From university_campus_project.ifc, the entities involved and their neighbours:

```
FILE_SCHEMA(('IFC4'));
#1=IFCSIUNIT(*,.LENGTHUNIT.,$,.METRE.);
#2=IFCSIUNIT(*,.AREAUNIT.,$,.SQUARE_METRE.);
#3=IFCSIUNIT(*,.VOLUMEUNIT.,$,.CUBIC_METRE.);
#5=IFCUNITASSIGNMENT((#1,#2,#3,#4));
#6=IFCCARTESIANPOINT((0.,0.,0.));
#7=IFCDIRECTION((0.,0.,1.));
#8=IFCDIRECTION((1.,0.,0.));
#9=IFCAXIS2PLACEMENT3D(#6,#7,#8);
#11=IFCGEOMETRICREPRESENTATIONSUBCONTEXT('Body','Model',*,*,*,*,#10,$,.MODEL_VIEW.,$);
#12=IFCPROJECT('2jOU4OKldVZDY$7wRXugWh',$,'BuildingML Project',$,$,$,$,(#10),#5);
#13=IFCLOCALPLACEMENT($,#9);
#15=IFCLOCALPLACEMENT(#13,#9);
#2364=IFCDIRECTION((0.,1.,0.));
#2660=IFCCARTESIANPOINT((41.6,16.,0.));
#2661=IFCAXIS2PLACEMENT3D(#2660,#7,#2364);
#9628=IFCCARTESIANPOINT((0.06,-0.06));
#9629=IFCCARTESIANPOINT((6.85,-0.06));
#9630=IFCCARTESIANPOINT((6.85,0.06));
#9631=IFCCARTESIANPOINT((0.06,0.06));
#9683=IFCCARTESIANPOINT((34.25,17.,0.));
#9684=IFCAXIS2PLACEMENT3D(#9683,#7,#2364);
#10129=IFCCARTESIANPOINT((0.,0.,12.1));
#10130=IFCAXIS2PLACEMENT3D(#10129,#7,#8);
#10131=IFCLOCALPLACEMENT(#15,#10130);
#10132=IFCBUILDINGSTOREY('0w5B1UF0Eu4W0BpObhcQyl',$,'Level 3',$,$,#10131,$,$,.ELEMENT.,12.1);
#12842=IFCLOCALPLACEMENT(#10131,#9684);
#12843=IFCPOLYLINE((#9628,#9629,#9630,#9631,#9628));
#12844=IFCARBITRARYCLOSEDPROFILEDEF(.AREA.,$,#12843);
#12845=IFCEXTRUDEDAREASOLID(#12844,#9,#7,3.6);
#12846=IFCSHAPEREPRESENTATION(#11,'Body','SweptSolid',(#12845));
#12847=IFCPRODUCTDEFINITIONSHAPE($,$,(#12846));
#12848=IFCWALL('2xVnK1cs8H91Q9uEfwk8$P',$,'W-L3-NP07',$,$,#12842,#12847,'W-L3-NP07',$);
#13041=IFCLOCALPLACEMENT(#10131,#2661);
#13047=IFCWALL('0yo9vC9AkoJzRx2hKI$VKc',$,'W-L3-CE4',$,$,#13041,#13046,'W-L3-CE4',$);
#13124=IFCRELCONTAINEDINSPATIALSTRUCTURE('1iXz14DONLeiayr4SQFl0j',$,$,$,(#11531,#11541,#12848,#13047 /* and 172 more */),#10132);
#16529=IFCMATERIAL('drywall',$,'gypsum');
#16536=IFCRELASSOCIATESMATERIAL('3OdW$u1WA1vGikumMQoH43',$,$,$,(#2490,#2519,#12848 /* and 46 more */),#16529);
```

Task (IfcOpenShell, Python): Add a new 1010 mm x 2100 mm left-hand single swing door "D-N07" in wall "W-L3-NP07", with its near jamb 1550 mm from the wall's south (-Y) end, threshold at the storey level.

```python
import numpy as np
import ifcopenshell
import ifcopenshell.api.feature
import ifcopenshell.api.geometry
import ifcopenshell.api.root
import ifcopenshell.api.spatial
import ifcopenshell.geom
import ifcopenshell.util.element
import ifcopenshell.util.placement
import ifcopenshell.util.representation
import ifcopenshell.util.shape
import ifcopenshell.util.unit

model = ifcopenshell.open("university_campus_project.ifc")
unit_scale = ifcopenshell.util.unit.calculate_unit_scale(model)
settings = ifcopenshell.geom.settings()


def volume(element):
    """Net volume in cubic metres, openings subtracted."""
    shape = ifcopenshell.geom.create_shape(settings, element)
    return ifcopenshell.util.shape.get_volume(shape.geometry)


wall = model.by_guid("2xVnK1cs8H91Q9uEfwk8$P")
storey = ifcopenshell.util.element.get_container(wall, ifc_class="IfcBuildingStorey")
context = ifcopenshell.util.representation.get_context(model, "Model", "Body", "MODEL_VIEW")
before = volume(wall)

width, height, from_end, sill = 1.01, 2.1, 1.55, 0.0  # metres

# The wall runs along its own X axis, and the end named is its -X end.
wall_shape = ifcopenshell.geom.create_shape(settings, wall)
x, y, z = ifcopenshell.util.shape.get_vertices(wall_shape.geometry).T
start = x.min() + from_end
face, thickness = float(y.min()), float(y.max() - y.min())
wall_matrix = ifcopenshell.util.placement.get_local_placement(wall.ObjectPlacement)
level = ifcopenshell.util.placement.get_local_placement(storey.ObjectPlacement)[2, 3]


def in_wall(x, y):
    """Placement at x, y metres in the wall's axes, at sill height."""
    matrix = wall_matrix.copy()
    matrix[:, 3] = wall_matrix @ np.array([x / unit_scale, y / unit_scale, 0.0, 1.0])
    matrix[2, 3] = level + sill / unit_scale
    return matrix


# Opening: a box that overshoots both wall faces by 50 mm.
opening = ifcopenshell.api.root.create_entity(model, ifc_class="IfcOpeningElement", predefined_type="OPENING")
box = ifcopenshell.api.geometry.add_wall_representation(
    model, context=context, length=width, height=height, thickness=thickness + 0.1
)
ifcopenshell.api.geometry.assign_representation(model, product=opening, representation=box)
ifcopenshell.api.geometry.edit_object_placement(model, product=opening, matrix=in_wall(start, face - 0.05), is_si=False)
ifcopenshell.api.feature.add_feature(model, feature=opening, element=wall)

door = ifcopenshell.api.root.create_entity(model, ifc_class="IfcDoor", name="D-N07", predefined_type="DOOR")
door.OverallWidth, door.OverallHeight = width / unit_scale, height / unit_scale
door.OperationType = "SINGLE_SWING_LEFT"
body = ifcopenshell.api.geometry.add_door_representation(
    model,
    context=context,
    overall_width=door.OverallWidth,
    overall_height=door.OverallHeight,
    operation_type="SINGLE_SWING_LEFT",
    lining_properties={"LiningDepth": thickness / unit_scale, "ThresholdDepth": thickness / unit_scale},
)
ifcopenshell.api.geometry.assign_representation(model, product=door, representation=body)
ifcopenshell.api.spatial.assign_container(model, products=[door], relating_structure=storey)
ifcopenshell.api.feature.add_filling(model, opening=opening, element=door)

# The lining spans the wall, so the door starts at the wall face.
ifcopenshell.api.geometry.edit_object_placement(model, product=door, matrix=in_wall(start, face), is_si=False)

after = volume(wall)

print(f"wall volume {before:.3f} -> {after:.3f} m3")

model.write("university_campus_project-out.ifc")
```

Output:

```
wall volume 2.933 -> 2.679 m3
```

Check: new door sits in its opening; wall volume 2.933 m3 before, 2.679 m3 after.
